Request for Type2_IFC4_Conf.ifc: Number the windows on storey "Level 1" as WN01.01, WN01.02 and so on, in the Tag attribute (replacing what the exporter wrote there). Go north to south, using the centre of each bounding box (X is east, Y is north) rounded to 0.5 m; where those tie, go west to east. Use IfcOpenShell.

First a look at what the model holds.

```python
import ifcopenshell
import ifcopenshell.util.element
import ifcopenshell.util.placement

model = ifcopenshell.open("Type2_IFC4_Conf.ifc")
print(model.schema)
storey = next(s for s in model.by_type("IfcBuildingStorey") if s.Name == "Level 1")
windows = [e for e in ifcopenshell.util.element.get_decomposition(storey) if e.is_a("IfcWindow")]
for e in sorted(windows, key=lambda e: e.id()):
    origin = ifcopenshell.util.placement.get_local_placement(e.ObjectPlacement)[:3, 3]
    print(e.id(), e.Tag, e.Name, origin.round(2) + 0.0, sep=" | ")
```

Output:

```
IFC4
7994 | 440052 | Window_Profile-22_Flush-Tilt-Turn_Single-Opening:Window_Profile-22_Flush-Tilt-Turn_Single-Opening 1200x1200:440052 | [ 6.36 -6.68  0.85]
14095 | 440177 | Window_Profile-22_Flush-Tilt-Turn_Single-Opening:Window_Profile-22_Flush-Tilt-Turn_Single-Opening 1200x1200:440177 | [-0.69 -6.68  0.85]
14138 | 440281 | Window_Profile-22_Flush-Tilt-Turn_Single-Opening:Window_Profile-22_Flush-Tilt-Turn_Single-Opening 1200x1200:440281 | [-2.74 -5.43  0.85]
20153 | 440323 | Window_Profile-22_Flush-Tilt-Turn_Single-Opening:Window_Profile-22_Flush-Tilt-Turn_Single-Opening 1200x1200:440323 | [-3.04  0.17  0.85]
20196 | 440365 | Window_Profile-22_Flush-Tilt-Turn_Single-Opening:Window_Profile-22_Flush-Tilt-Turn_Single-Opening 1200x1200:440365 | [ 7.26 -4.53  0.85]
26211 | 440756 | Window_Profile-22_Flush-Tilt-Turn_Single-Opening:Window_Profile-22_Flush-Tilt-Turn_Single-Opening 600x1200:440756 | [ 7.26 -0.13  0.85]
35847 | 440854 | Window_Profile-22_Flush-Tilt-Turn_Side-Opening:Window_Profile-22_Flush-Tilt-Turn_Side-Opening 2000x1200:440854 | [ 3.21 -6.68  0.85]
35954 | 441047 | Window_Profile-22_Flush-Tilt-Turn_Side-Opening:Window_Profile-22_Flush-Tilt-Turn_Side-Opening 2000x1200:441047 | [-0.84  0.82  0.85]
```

```python
import ifcopenshell
import ifcopenshell.geom
import ifcopenshell.util.element
import ifcopenshell.util.shape

model = ifcopenshell.open("Type2_IFC4_Conf.ifc")
settings = ifcopenshell.geom.settings()
settings.set("use-world-coords", True)


def centre(element):
    shape = ifcopenshell.geom.create_shape(settings, element)
    return ifcopenshell.util.shape.get_bbox_centroid(shape.geometry)


storey = next(s for s in model.by_type("IfcBuildingStorey") if s.Name == "Level 1")
windows = [e for e in ifcopenshell.util.element.get_decomposition(storey) if e.is_a("IfcWindow")]

# Insertion points can sit at a corner or the storey origin, so sort by the geometry (in metres).
centres = {e: centre(e) for e in windows}
windows.sort(key=lambda e: (-round(centres[e][1] / 0.5), centres[e][0]))

for i, e in enumerate(windows, start=1):
    number = f"WN01.{i:02d}"
    e.Tag = number
    print(e.id(), number)

model.write("Type2_IFC4_Conf_v2.ifc")
```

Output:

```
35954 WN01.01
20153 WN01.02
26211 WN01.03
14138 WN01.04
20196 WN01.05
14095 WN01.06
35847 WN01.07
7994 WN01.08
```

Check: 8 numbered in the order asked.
